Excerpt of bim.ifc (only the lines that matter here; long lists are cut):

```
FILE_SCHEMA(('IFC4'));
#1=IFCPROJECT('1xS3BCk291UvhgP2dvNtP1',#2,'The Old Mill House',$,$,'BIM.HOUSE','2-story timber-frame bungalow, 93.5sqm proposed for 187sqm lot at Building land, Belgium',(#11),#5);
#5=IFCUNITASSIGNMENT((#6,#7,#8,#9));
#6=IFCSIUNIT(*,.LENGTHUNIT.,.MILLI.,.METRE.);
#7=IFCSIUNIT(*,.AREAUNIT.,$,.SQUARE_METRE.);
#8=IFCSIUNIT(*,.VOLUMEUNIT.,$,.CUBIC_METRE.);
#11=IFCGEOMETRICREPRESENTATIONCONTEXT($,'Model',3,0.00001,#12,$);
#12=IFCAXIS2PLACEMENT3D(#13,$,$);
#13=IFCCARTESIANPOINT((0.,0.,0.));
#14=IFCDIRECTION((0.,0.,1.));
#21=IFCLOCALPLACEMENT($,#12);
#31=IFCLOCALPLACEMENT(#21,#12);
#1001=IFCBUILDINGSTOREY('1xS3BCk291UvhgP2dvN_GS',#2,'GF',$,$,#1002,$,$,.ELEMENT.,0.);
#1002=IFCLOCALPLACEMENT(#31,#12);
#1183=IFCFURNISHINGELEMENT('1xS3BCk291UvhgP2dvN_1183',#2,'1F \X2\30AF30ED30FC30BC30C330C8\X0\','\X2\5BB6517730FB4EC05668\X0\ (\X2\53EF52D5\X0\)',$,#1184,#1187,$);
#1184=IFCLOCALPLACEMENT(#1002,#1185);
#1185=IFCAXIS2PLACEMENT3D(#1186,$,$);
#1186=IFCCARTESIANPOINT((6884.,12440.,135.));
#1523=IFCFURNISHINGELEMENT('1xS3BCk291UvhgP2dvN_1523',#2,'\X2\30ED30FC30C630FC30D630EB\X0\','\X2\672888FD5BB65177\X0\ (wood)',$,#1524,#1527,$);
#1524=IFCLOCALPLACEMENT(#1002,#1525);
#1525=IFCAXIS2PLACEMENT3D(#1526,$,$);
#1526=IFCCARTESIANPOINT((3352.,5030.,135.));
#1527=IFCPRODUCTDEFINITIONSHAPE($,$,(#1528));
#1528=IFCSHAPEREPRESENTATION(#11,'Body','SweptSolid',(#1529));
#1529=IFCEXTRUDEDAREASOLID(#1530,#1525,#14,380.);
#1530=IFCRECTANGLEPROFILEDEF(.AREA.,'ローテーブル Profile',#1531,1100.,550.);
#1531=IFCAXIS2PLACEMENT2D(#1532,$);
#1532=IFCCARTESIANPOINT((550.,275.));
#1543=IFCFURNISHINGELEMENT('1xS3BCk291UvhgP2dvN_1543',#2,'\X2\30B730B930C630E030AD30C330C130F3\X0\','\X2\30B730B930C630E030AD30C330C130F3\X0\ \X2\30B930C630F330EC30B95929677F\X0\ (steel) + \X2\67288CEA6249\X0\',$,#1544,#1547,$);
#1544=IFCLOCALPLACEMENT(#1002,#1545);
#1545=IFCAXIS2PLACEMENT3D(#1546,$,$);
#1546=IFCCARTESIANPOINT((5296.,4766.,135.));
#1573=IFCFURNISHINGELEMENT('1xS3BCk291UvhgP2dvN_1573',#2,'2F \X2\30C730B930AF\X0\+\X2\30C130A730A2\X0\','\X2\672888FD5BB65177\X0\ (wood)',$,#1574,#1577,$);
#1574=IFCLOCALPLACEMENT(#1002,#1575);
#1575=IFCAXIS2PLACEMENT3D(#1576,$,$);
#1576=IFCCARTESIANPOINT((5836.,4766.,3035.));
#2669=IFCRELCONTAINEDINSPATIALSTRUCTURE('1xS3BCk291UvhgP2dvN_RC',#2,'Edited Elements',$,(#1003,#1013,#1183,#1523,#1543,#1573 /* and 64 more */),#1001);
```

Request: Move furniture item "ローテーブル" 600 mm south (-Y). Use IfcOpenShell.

```python
import ifcopenshell
import ifcopenshell.api.geometry
import ifcopenshell.util.placement
import ifcopenshell.util.unit

model = ifcopenshell.open("bim.ifc")
unit_scale = ifcopenshell.util.unit.calculate_unit_scale(model)

item = model.by_id(1523)
matrix = ifcopenshell.util.placement.get_local_placement(item.ObjectPlacement)
matrix[1, 3] -= 0.6 / unit_scale
ifcopenshell.api.geometry.edit_object_placement(model, product=item, matrix=matrix, is_si=False)

print(ifcopenshell.util.placement.get_local_placement(item.ObjectPlacement).round(3) + 0.0)

model.write("bim_rev.ifc")
```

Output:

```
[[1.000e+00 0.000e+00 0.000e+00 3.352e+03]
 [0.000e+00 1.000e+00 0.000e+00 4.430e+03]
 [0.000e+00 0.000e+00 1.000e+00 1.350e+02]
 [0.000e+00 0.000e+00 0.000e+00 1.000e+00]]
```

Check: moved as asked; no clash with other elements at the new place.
